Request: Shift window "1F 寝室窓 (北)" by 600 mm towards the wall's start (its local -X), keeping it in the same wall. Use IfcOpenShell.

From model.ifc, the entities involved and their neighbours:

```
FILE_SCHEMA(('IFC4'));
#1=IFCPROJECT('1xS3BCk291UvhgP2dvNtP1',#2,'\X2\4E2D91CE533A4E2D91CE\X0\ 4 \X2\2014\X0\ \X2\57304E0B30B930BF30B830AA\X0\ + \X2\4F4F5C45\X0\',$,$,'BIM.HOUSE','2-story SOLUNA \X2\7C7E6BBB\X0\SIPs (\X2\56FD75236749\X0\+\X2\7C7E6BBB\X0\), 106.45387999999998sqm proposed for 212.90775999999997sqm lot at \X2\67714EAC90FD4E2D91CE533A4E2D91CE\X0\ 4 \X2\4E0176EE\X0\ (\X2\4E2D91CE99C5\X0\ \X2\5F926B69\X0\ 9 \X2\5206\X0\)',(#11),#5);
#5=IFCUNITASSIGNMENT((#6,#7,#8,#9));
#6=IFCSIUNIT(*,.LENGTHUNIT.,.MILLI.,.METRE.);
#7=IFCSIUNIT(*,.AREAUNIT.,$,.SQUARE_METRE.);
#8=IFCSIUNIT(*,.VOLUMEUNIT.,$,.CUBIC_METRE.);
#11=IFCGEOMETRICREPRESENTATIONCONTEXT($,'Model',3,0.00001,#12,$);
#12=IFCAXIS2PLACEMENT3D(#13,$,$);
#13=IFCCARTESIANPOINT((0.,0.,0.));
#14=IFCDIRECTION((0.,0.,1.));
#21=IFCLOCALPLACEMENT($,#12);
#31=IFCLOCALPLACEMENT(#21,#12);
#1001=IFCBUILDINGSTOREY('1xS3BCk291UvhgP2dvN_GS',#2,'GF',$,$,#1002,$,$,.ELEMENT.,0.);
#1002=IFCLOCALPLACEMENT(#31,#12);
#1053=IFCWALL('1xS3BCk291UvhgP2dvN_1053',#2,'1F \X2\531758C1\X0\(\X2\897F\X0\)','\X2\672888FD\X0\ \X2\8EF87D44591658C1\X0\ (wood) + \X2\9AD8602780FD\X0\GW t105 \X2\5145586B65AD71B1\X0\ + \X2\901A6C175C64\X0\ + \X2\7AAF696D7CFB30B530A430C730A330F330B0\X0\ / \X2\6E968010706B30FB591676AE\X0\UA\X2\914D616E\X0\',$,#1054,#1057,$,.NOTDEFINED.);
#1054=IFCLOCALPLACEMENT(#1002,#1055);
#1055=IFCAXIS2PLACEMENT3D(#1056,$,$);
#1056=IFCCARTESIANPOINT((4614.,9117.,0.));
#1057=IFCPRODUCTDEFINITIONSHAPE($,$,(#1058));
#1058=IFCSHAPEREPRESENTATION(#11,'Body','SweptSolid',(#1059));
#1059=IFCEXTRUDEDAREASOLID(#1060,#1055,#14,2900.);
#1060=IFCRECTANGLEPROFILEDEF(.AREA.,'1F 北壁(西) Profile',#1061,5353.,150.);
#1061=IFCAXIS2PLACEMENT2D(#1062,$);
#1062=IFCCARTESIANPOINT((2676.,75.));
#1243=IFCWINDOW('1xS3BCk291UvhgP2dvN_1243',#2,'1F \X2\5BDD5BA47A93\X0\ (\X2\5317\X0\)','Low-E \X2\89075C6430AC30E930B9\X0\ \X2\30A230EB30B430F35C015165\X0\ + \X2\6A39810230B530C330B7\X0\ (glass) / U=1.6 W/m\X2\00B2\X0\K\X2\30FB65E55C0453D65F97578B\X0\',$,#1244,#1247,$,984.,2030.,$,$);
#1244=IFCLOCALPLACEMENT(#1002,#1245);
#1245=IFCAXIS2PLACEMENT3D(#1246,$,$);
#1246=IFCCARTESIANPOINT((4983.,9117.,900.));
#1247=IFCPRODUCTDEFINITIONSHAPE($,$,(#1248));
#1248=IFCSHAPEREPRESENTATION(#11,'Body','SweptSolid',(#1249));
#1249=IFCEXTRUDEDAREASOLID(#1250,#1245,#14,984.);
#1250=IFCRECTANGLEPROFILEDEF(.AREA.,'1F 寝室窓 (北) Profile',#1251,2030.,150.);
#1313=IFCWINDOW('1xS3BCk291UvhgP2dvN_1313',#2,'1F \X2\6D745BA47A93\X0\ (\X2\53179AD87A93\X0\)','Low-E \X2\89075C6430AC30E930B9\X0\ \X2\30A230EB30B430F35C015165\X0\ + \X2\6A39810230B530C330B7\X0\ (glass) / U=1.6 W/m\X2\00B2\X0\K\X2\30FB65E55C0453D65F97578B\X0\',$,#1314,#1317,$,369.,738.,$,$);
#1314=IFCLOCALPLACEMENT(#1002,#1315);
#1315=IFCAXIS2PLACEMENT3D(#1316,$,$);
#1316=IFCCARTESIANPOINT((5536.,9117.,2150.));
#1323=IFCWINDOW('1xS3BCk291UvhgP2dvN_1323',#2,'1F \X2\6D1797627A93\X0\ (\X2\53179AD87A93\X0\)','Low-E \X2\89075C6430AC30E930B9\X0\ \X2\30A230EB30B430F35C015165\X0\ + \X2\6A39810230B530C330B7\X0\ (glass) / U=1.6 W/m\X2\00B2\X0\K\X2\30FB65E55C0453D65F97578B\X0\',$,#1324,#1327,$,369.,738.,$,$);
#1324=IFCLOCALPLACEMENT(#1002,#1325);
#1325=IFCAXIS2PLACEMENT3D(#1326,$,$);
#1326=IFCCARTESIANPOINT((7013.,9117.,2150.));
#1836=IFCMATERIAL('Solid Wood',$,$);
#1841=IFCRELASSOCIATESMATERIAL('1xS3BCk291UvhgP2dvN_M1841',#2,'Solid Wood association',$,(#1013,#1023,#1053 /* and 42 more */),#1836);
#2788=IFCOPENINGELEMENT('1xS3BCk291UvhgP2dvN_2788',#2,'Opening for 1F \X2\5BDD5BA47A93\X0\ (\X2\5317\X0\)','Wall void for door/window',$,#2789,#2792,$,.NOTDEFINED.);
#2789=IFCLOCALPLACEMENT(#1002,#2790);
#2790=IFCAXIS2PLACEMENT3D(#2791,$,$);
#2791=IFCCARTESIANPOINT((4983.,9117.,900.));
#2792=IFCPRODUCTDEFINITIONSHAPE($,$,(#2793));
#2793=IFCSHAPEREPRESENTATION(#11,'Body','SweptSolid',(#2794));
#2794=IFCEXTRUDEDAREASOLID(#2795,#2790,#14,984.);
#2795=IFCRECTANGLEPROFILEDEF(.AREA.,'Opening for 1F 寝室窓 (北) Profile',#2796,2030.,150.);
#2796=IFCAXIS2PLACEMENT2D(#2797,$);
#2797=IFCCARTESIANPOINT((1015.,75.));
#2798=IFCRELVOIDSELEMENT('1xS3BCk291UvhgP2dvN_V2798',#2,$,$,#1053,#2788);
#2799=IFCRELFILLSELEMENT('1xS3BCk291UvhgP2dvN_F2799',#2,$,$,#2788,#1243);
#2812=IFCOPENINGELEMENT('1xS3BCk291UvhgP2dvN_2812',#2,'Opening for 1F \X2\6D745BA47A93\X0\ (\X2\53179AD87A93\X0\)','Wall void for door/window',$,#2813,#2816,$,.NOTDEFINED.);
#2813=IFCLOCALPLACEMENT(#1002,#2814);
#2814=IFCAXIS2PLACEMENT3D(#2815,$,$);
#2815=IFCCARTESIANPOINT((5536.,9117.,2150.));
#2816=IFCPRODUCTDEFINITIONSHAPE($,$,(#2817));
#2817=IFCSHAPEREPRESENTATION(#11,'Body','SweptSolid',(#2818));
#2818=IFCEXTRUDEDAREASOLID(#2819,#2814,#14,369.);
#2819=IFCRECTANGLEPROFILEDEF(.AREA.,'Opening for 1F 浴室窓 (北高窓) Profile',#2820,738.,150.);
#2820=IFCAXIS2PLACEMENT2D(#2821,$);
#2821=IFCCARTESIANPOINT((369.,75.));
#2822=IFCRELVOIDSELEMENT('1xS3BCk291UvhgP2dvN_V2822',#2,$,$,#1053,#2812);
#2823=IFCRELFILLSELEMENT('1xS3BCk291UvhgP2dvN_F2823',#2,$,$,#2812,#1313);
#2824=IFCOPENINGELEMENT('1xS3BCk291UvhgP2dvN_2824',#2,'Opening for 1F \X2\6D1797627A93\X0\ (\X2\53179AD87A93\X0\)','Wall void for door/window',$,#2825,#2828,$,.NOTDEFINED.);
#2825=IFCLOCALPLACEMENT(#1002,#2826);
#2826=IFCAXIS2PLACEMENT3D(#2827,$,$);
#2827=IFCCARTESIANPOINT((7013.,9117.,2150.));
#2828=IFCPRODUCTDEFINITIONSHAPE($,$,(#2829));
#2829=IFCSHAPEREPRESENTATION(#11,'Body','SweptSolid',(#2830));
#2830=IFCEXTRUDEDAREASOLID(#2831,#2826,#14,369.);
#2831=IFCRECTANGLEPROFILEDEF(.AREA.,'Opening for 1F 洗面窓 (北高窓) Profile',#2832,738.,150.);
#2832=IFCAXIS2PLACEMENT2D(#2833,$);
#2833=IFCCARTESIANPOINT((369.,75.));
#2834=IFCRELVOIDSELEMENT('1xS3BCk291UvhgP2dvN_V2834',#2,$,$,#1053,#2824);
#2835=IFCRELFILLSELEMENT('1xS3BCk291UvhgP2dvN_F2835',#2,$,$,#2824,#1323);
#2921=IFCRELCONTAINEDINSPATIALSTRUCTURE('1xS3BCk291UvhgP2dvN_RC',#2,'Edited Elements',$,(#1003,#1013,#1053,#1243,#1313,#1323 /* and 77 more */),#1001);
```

```python
import ifcopenshell
import ifcopenshell.api.geometry
import ifcopenshell.util.placement

model = ifcopenshell.open("model.ifc")

window = model.by_guid("1xS3BCk291UvhgP2dvN_1243")
opening = window.FillsVoids[0].RelatingOpeningElement
wall = opening.VoidsElements[0].RelatingBuildingElement

wall_matrix = ifcopenshell.util.placement.get_local_placement(wall.ObjectPlacement)
shift = wall_matrix[:3, 0] * -600.0
before = ifcopenshell.util.placement.get_local_placement(window.ObjectPlacement)[:3, 3].copy()

# The window is not placed relative to its opening, so move both.
for product in (opening, window):
    matrix = ifcopenshell.util.placement.get_local_placement(product.ObjectPlacement)
    matrix[:3, 3] += shift
    ifcopenshell.api.geometry.edit_object_placement(model, product=product, matrix=matrix, is_si=False)

after = ifcopenshell.util.placement.get_local_placement(window.ObjectPlacement)[:3, 3]
print("window moved by", (after - before).round(3) + 0.0)

model.write("model-out.ifc")
```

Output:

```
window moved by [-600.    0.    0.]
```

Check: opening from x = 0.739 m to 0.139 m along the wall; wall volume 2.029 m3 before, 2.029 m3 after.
